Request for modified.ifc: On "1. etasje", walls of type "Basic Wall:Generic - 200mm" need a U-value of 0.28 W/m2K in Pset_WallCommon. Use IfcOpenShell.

First a look at what the model holds.

```python
import ifcopenshell
import ifcopenshell.util.element

model = ifcopenshell.open("modified.ifc")
print(model.schema)
storey = next(s for s in model.by_type("IfcBuildingStorey") if s.Name == "1. etasje")
walls = [e for e in ifcopenshell.util.element.get_decomposition(storey) if e.is_a("IfcWall")]
seen = {}
for e in walls:
    element_type = ifcopenshell.util.element.get_type(e)
    key = (element_type.Name if element_type != e and element_type else None, ifcopenshell.util.element.get_pset(e, "Pset_WallCommon", "ThermalTransmittance"))
    seen[key] = seen.get(key, 0) + 1
for (name, value), count in sorted(seen.items(), key=str):
    print(count, "x", name, "|", value)
```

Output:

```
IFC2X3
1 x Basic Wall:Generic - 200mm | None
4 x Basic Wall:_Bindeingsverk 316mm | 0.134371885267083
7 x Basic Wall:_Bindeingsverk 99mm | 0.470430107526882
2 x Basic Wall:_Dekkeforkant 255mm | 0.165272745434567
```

```python
import ifcopenshell
import ifcopenshell.api.pset
import ifcopenshell.util.element

model = ifcopenshell.open("modified.ifc")

storey = next(s for s in model.by_type("IfcBuildingStorey") if s.Name == "1. etasje")
walls = [e for e in ifcopenshell.util.element.get_decomposition(storey) if e.is_a("IfcWall")]

count = 0
for e in walls:
    element_type = ifcopenshell.util.element.get_type(e)
    if element_type in (None, e) or element_type.Name != "Basic Wall:Generic - 200mm":
        continue
    # add_pset returns the element's existing set when there is one.
    pset = ifcopenshell.api.pset.add_pset(model, product=e, name="Pset_WallCommon")
    ifcopenshell.api.pset.edit_pset(model, pset=pset, properties={"ThermalTransmittance": 0.28})
    count += 1

print(count, "walls updated")

model.write("modified_updated.ifc")
```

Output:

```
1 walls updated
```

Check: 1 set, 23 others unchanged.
